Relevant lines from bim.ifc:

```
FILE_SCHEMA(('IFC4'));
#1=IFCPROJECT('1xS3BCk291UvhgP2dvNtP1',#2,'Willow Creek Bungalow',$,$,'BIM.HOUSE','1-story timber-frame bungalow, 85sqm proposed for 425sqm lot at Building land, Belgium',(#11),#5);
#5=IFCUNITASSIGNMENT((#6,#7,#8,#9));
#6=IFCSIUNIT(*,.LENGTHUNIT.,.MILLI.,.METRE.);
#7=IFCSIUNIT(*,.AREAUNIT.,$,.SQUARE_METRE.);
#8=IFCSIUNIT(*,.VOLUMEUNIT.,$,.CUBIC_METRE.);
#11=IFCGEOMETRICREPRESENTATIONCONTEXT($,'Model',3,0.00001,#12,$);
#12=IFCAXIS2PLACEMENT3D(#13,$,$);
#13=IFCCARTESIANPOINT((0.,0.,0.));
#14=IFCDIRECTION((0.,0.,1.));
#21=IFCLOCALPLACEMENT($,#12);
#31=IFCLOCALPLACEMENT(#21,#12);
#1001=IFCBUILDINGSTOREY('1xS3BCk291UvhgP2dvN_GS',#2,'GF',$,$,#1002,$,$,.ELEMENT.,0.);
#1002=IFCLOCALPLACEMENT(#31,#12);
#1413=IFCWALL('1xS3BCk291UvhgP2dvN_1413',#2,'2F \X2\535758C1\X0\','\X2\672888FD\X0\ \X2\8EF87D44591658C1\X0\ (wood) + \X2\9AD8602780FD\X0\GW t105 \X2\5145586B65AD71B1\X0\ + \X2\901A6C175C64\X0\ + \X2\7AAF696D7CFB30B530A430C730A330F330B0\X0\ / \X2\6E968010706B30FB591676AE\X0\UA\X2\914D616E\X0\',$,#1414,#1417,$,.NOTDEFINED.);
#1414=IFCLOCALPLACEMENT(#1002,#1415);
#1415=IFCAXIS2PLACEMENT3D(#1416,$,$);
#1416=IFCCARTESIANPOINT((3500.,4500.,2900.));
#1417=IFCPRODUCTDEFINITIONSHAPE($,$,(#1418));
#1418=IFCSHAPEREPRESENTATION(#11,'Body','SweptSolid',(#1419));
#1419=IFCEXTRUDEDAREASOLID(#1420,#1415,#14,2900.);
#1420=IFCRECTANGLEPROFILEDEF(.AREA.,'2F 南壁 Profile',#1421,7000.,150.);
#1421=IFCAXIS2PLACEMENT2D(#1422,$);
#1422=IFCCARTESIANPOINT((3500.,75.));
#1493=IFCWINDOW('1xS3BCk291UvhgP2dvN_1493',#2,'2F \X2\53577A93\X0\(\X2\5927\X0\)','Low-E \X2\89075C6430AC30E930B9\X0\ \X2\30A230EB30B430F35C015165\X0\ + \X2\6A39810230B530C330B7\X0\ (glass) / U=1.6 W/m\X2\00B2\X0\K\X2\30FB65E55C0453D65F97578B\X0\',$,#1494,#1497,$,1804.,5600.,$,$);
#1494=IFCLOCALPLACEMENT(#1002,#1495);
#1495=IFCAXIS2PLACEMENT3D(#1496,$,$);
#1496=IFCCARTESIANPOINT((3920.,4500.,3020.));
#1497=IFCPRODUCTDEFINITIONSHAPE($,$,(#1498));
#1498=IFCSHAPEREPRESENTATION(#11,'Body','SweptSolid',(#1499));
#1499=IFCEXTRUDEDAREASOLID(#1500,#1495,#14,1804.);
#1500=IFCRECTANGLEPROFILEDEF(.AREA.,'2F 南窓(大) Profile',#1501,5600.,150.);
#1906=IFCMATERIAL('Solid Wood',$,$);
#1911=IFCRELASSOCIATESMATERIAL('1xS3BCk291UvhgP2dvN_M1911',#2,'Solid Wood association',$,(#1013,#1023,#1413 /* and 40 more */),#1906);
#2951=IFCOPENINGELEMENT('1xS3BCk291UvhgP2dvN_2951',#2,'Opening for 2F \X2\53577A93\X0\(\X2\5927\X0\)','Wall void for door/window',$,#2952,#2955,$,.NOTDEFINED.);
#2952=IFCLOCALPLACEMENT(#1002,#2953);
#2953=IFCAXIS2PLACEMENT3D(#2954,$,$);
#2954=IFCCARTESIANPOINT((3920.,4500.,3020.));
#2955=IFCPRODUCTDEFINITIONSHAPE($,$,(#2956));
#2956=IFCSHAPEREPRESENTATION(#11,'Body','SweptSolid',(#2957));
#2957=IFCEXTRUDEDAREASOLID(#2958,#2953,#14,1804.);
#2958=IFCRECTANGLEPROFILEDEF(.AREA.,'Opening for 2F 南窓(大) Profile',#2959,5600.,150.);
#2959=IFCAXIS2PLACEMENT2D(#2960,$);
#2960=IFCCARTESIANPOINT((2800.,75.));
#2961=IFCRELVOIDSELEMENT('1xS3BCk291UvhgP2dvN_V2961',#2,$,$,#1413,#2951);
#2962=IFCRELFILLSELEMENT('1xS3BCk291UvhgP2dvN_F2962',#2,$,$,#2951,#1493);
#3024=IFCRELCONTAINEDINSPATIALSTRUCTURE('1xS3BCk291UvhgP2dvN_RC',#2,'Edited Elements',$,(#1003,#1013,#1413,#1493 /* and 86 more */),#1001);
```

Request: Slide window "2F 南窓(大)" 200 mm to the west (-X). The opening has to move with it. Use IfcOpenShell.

```python
import ifcopenshell
import ifcopenshell.api.geometry
import ifcopenshell.util.placement
import ifcopenshell.util.unit

model = ifcopenshell.open("bim.ifc")
unit_scale = ifcopenshell.util.unit.calculate_unit_scale(model)

window = model.by_guid("1xS3BCk291UvhgP2dvN_1493")
opening = window.FillsVoids[0].RelatingOpeningElement
wall = opening.VoidsElements[0].RelatingBuildingElement

wall_matrix = ifcopenshell.util.placement.get_local_placement(wall.ObjectPlacement)
shift = wall_matrix[:3, 0] * -0.2 / unit_scale
before = ifcopenshell.util.placement.get_local_placement(window.ObjectPlacement)[:3, 3].copy()

# The window is not placed relative to its opening, so move both.
for product in (opening, window):
    matrix = ifcopenshell.util.placement.get_local_placement(product.ObjectPlacement)
    matrix[:3, 3] += shift
    ifcopenshell.api.geometry.edit_object_placement(model, product=product, matrix=matrix, is_si=False)

after = ifcopenshell.util.placement.get_local_placement(window.ObjectPlacement)[:3, 3]
print("window moved by", (after - before).round(3) + 0.0)

model.write("bim_v2.ifc")
```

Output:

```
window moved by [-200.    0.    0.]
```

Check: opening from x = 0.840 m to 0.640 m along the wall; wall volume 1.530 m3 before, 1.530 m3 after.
